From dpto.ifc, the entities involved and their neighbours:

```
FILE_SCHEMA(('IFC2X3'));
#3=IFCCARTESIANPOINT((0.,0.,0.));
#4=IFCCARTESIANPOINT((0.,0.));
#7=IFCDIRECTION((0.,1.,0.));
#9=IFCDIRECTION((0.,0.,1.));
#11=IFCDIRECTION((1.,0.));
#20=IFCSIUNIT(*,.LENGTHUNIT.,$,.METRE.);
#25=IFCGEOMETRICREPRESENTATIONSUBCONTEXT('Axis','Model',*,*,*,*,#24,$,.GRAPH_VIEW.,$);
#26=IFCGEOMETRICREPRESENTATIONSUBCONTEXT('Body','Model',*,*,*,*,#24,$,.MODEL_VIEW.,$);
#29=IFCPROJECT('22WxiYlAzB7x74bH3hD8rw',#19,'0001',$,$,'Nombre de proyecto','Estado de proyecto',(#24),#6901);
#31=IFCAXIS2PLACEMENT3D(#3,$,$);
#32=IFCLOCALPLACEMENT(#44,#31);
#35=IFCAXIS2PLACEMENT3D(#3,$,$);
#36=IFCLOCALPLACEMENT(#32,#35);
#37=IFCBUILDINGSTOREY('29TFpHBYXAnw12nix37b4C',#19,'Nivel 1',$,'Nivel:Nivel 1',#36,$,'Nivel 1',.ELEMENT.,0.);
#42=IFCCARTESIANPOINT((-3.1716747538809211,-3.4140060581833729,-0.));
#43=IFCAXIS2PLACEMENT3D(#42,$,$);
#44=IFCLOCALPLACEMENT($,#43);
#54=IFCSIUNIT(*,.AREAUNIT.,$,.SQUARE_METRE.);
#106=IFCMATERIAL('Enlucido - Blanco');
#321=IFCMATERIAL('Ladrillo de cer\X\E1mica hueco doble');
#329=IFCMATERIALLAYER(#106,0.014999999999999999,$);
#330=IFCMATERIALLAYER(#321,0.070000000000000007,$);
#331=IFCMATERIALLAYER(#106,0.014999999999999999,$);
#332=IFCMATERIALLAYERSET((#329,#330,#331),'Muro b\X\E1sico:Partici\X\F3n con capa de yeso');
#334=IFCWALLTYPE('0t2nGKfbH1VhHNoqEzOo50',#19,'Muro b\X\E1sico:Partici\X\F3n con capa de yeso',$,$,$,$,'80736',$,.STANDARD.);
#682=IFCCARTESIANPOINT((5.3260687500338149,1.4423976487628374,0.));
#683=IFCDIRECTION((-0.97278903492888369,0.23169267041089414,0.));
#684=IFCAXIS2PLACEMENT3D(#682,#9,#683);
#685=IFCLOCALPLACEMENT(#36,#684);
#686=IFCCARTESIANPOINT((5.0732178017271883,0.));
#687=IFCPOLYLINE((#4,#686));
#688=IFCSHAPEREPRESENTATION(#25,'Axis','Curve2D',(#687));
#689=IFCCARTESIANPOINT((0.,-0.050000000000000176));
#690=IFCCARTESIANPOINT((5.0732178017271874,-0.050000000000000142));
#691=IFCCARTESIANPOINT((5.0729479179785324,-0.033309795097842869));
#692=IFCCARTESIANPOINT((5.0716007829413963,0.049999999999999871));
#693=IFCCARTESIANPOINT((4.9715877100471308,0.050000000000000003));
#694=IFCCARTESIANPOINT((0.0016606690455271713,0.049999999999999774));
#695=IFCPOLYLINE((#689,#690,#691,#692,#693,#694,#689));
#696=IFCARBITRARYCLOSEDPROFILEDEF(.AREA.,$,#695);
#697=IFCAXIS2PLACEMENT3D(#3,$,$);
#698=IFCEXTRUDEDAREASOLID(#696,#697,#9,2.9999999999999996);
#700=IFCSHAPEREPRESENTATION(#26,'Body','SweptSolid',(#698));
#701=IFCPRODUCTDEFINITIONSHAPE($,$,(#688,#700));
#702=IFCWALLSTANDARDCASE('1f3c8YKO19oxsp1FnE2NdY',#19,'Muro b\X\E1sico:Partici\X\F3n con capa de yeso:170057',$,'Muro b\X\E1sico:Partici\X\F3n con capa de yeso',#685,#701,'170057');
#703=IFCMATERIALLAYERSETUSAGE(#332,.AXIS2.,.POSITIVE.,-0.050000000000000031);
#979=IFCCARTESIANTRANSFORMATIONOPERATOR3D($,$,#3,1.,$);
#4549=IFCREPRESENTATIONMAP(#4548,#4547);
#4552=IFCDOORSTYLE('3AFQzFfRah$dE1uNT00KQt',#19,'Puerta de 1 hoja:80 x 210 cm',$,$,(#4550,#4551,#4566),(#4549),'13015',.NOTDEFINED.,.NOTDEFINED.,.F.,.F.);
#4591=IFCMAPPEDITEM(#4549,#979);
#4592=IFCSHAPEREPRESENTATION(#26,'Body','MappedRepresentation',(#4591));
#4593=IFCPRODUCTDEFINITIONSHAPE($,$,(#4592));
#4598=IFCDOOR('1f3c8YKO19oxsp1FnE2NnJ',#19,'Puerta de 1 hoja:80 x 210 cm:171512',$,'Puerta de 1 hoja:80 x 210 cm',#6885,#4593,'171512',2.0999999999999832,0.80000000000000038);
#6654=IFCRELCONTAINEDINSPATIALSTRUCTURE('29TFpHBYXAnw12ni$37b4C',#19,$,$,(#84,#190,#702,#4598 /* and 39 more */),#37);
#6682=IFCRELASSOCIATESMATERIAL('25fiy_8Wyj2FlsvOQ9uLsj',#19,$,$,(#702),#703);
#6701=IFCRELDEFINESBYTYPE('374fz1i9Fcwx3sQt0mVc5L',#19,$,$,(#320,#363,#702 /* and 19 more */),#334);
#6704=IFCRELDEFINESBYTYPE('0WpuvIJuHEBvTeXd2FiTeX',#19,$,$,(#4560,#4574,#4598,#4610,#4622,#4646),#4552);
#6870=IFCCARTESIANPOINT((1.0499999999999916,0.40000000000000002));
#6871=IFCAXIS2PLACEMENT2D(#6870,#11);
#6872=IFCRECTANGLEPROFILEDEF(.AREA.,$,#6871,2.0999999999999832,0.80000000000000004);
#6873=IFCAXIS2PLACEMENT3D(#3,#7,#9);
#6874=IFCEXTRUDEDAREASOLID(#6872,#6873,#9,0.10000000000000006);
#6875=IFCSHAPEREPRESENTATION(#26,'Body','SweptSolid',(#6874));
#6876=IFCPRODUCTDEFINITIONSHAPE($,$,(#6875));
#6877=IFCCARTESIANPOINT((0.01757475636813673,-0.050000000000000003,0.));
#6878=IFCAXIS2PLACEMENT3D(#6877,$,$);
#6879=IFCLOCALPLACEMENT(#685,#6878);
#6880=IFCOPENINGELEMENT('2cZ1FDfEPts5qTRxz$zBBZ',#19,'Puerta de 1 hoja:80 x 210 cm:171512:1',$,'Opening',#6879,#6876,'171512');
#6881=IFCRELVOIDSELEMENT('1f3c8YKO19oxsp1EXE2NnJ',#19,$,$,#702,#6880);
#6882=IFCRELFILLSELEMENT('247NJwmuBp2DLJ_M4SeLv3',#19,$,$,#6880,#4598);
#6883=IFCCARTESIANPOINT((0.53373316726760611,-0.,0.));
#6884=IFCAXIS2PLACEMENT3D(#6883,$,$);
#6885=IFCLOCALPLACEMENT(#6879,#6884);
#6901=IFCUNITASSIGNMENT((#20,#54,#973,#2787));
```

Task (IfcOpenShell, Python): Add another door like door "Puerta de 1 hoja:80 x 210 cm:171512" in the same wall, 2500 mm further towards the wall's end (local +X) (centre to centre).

```python
import ifcopenshell
import ifcopenshell.api.feature
import ifcopenshell.api.geometry
import ifcopenshell.api.root
import ifcopenshell.geom
import ifcopenshell.util.element
import ifcopenshell.util.placement
import ifcopenshell.util.shape

model = ifcopenshell.open("dpto.ifc")
settings = ifcopenshell.geom.settings()


def volume(element):
    """Net volume in cubic metres, openings subtracted."""
    shape = ifcopenshell.geom.create_shape(settings, element)
    return ifcopenshell.util.shape.get_volume(shape.geometry)


def reuse_history(source, copy):
    """copy_class also copies each property set's owner history, people and application; keep the originals."""
    for rel in copy.IsDefinedBy:
        if rel.is_a("IfcRelDefinesByProperties") and (history := rel.RelatingPropertyDefinition.OwnerHistory):
            rel.RelatingPropertyDefinition.OwnerHistory = source.OwnerHistory
            ifcopenshell.util.element.remove_deep2(model, history)


door = model.by_guid("1f3c8YKO19oxsp1FnE2NnJ")
opening = door.FillsVoids[0].RelatingOpeningElement
wall = opening.VoidsElements[0].RelatingBuildingElement
before = volume(wall)
shift = ifcopenshell.util.placement.get_local_placement(wall.ObjectPlacement)[:3, 0] * 2.5

# copy_class copies the void relationship, type, container and properties, but no geometry.
new_opening = ifcopenshell.api.root.copy_class(model, product=opening)
new_opening.Representation = ifcopenshell.util.element.copy_deep(
    model, opening.Representation, exclude=["IfcGeometricRepresentationContext", "IfcRepresentationMap"]
)
new_opening.Name = "Puerta de 1 hoja:80 x 210 cm"
new_opening.Tag = None
new_door = ifcopenshell.api.root.copy_class(model, product=door)
new_door.Representation = ifcopenshell.util.element.copy_deep(
    model, door.Representation, exclude=["IfcGeometricRepresentationContext", "IfcRepresentationMap"]
)
new_door.Name = "Puerta de 1 hoja:80 x 210 cm"
new_door.Tag = None
reuse_history(door, new_door)
fills = ifcopenshell.api.feature.add_filling(model, opening=new_opening, element=new_door)
fills.OwnerHistory = new_door.OwnerHistory  # required in IFC2X3

for old, new in ((opening, new_opening), (door, new_door)):
    matrix = ifcopenshell.util.placement.get_local_placement(old.ObjectPlacement)
    matrix[:3, 3] += shift
    ifcopenshell.api.geometry.edit_object_placement(model, product=new, matrix=matrix, is_si=False)

after = volume(wall)

print(f"wall volume {before:.3f} -> {after:.3f} m3")

model.write("dpto_v2.ifc")
```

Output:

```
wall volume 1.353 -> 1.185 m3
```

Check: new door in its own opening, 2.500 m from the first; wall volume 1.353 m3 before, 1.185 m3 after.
